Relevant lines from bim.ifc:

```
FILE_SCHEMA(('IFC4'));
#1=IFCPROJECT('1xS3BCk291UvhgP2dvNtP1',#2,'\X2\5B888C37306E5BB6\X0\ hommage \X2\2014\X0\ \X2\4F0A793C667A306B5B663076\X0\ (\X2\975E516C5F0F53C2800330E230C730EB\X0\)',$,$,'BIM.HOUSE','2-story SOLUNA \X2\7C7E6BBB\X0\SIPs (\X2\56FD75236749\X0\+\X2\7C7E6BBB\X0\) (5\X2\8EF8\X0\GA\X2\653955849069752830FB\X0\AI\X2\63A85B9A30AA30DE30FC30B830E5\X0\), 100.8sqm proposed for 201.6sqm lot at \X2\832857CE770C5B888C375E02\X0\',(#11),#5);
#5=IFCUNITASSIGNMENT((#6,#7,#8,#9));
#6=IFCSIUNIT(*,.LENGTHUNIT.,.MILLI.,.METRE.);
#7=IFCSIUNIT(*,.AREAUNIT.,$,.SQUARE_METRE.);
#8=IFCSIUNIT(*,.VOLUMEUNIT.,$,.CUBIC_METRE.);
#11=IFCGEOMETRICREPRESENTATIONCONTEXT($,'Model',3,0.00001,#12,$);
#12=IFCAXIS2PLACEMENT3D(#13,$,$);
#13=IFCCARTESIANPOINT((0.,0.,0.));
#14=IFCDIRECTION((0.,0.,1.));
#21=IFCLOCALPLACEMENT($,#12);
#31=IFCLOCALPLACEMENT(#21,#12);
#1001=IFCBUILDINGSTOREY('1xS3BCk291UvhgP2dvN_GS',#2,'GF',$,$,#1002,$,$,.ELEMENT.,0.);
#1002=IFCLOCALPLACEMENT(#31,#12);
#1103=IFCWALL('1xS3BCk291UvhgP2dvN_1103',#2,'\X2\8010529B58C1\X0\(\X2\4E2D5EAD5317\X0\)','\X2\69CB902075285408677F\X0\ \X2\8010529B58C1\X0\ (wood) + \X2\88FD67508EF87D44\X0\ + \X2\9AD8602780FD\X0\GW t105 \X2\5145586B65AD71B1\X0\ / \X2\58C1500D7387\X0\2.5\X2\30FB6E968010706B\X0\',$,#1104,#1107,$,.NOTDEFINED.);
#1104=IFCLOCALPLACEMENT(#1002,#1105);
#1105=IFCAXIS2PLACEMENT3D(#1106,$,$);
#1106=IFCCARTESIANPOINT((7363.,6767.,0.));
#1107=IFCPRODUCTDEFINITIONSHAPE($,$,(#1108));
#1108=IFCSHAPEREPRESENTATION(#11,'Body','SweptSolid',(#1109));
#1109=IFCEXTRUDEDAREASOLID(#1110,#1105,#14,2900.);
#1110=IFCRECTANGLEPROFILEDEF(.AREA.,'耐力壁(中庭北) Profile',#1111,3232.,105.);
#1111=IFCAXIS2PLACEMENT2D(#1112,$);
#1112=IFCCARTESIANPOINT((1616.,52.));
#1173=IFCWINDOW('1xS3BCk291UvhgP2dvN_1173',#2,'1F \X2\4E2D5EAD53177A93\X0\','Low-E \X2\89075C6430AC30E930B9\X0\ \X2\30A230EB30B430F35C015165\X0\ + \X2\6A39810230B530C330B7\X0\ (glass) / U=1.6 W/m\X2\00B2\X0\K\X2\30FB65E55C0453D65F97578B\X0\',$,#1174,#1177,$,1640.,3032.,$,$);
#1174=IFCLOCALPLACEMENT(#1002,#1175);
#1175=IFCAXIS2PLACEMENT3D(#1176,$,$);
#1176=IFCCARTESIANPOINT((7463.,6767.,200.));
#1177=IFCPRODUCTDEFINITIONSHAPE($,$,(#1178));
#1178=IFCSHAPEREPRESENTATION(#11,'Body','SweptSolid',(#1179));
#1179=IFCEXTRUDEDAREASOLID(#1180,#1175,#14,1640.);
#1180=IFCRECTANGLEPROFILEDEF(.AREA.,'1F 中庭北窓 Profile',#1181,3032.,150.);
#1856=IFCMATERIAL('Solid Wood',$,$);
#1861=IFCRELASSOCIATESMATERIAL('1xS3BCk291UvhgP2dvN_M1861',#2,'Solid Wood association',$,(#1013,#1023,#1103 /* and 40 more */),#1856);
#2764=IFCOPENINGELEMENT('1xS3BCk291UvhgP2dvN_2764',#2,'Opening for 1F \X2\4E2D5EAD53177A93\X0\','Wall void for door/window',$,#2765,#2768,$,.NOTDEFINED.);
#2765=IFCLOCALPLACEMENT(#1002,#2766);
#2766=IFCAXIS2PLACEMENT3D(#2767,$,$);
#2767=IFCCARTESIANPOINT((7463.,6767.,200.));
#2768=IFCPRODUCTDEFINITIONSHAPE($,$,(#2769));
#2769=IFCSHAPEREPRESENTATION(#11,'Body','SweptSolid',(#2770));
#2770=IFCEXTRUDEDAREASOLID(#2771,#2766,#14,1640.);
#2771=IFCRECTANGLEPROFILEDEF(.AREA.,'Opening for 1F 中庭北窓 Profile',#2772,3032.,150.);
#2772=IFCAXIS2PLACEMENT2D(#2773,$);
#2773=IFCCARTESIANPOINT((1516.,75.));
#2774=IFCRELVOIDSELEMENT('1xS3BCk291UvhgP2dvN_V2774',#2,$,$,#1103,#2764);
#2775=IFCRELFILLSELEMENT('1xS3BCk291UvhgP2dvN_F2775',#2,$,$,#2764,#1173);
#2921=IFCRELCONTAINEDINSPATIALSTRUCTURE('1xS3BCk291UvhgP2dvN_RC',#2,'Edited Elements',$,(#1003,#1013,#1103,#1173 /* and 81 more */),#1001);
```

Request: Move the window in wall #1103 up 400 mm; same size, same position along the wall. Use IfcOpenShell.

```python
import numpy as np
import ifcopenshell
import ifcopenshell.api.geometry
import ifcopenshell.util.placement
import ifcopenshell.util.unit

model = ifcopenshell.open("bim.ifc")
unit_scale = ifcopenshell.util.unit.calculate_unit_scale(model)

window = model.by_id(1173)
opening = window.FillsVoids[0].RelatingOpeningElement
dz = 400.0

shift = np.array([0.0, 0.0, dz])
# The window is not placed relative to its opening, so move both.
for product in (opening, window):
    matrix = ifcopenshell.util.placement.get_local_placement(product.ObjectPlacement)
    matrix[:3, 3] += shift
    ifcopenshell.api.geometry.edit_object_placement(model, product=product, matrix=matrix, is_si=False)

print(f"moved by {dz * unit_scale:+.3f} m")

model.write("bim_edited.ifc")
```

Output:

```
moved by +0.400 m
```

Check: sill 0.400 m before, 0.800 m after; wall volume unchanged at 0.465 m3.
